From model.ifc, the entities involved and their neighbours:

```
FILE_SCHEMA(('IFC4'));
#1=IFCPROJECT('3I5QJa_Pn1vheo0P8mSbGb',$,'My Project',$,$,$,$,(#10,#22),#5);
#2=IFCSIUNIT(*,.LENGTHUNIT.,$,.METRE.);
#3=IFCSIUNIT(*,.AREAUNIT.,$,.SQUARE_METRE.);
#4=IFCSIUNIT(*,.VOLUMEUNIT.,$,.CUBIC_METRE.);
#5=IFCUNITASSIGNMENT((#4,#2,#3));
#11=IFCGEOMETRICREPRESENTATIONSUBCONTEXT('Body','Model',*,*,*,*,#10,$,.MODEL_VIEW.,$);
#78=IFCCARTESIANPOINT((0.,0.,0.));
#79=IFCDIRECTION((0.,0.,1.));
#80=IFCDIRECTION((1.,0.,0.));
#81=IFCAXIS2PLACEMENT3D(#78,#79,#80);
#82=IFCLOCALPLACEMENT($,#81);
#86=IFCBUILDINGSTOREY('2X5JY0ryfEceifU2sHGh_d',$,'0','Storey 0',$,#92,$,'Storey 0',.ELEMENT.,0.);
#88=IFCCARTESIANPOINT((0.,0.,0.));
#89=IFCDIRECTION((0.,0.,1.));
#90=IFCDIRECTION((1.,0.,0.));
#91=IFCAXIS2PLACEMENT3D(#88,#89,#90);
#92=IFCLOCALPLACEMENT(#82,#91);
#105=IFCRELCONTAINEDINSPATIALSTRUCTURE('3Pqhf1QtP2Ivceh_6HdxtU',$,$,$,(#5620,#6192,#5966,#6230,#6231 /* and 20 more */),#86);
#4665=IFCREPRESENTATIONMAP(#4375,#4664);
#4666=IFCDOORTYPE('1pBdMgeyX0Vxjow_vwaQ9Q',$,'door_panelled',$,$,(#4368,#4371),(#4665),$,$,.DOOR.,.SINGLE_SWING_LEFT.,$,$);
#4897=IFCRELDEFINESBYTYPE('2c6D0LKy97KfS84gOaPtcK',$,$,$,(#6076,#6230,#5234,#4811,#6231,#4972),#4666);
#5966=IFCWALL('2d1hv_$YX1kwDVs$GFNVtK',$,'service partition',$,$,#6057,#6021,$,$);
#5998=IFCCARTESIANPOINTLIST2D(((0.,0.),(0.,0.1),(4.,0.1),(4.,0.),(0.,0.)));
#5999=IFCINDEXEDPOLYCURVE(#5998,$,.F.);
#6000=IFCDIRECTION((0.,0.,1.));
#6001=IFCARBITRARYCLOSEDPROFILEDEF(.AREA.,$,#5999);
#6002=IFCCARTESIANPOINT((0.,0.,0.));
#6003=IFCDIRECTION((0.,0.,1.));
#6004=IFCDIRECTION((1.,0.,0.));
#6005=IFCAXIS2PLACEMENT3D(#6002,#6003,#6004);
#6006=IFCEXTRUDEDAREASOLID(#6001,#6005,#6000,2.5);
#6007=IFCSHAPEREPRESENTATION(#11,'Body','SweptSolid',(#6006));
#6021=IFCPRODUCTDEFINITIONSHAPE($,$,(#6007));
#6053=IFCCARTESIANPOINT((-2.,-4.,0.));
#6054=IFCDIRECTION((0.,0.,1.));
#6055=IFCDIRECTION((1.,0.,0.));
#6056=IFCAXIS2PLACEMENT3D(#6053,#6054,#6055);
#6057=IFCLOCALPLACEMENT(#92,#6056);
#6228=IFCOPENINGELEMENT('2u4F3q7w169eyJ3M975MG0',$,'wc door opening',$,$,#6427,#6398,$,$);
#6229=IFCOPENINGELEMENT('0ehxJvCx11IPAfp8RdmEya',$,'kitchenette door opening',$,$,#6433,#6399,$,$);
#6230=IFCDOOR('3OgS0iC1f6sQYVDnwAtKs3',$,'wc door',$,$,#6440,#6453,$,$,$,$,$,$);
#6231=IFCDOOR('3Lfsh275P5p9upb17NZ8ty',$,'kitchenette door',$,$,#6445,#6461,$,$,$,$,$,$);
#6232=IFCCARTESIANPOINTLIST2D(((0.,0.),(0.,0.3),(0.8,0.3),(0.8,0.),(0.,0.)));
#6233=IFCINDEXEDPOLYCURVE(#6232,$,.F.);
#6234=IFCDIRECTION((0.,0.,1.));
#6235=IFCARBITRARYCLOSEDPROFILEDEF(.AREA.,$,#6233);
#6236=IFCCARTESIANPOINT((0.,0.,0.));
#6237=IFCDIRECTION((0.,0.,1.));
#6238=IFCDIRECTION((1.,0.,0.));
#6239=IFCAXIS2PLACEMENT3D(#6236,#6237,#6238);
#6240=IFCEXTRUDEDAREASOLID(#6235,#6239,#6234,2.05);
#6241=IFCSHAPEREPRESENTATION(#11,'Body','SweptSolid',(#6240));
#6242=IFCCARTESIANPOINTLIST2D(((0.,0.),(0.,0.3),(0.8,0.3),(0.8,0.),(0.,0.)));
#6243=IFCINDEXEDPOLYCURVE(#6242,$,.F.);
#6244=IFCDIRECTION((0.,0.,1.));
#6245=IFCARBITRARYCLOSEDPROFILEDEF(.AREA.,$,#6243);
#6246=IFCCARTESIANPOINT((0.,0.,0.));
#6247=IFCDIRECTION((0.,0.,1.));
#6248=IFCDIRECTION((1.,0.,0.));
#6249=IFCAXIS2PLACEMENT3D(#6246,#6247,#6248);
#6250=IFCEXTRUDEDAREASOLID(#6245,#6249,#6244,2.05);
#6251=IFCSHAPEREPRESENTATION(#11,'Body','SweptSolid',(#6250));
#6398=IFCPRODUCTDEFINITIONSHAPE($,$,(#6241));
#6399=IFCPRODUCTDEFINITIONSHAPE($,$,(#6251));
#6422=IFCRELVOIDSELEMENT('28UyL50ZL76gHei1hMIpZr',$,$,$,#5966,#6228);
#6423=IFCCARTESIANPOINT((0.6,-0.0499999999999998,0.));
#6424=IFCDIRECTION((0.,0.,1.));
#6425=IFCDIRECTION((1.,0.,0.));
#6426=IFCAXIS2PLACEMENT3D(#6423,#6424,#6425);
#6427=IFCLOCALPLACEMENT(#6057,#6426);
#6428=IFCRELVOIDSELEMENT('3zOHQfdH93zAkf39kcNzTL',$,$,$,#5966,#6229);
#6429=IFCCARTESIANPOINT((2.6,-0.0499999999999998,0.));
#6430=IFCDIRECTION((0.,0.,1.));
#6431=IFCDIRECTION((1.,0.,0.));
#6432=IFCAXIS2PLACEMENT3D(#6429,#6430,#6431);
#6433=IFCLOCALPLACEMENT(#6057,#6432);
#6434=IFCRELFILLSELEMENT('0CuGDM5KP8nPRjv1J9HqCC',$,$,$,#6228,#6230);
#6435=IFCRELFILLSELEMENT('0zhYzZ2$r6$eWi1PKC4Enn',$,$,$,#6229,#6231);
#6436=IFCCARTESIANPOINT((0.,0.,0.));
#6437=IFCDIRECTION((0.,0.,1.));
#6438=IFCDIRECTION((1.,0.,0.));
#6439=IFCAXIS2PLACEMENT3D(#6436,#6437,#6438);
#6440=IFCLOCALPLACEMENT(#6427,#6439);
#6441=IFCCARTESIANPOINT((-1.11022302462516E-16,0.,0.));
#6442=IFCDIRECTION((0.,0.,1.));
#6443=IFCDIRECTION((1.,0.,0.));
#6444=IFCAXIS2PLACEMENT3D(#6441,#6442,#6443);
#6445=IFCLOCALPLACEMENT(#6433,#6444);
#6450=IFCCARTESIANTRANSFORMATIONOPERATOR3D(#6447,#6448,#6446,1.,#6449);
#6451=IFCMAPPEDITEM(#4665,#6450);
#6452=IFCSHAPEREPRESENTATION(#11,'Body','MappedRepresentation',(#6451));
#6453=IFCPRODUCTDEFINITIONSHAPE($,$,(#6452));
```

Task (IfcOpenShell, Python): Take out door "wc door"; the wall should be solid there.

```python
import ifcopenshell
import ifcopenshell.api.feature
import ifcopenshell.api.root
import ifcopenshell.geom
import ifcopenshell.util.shape

model = ifcopenshell.open("model.ifc")
settings = ifcopenshell.geom.settings()


def volume(element):
    """Net volume in cubic metres, openings subtracted."""
    shape = ifcopenshell.geom.create_shape(settings, element)
    return ifcopenshell.util.shape.get_volume(shape.geometry)


door = model.by_guid("3OgS0iC1f6sQYVDnwAtKs3")
opening = door.FillsVoids[0].RelatingOpeningElement
wall = opening.VoidsElements[0].RelatingBuildingElement
before = volume(wall)

ifcopenshell.api.root.remove_product(model, product=door)
ifcopenshell.api.feature.remove_feature(model, feature=opening)

after = volume(wall)

print(f"wall volume {before:.3f} -> {after:.3f} m3")

model.write("model_edited.ifc")
```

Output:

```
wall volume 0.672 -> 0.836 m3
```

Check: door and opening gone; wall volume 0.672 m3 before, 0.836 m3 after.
